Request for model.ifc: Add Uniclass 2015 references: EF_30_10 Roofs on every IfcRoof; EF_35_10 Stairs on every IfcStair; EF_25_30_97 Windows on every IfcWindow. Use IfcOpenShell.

First a look at what the model holds.

```python
import ifcopenshell

model = ifcopenshell.open("model.ifc")
print(model.schema)
print("classifications:", [c.Name for c in model.by_type("IfcClassification")])
for ifc_class in ("IfcDoor", "IfcRoof", "IfcStair", "IfcWall", "IfcWindow"):
    print(ifc_class, len(model.by_type(ifc_class)))
```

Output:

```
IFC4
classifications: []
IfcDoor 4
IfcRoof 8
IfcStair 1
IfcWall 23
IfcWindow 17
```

```python
import ifcopenshell
import ifcopenshell.api.classification

model = ifcopenshell.open("model.ifc")

system = ifcopenshell.api.classification.add_classification(model, classification="Uniclass 2015")

codes = {
    "IfcRoof": ("EF_30_10", "Roofs"),
    "IfcStair": ("EF_35_10", "Stairs"),
    "IfcWindow": ("EF_25_30_97", "Windows"),
}
for ifc_class, (code, name) in codes.items():
    products = model.by_type(ifc_class)
    ifcopenshell.api.classification.add_reference(
        model, products=products, classification=system, identification=code, name=name
    )
    print(code, len(products))

model.write("model_updated.ifc")
```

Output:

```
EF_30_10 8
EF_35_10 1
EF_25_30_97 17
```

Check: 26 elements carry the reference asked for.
